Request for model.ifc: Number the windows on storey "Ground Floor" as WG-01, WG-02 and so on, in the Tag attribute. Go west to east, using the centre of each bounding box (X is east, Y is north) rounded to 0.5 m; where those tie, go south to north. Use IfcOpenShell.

First a look at what the model holds.

```python
import ifcopenshell
import ifcopenshell.util.element
import ifcopenshell.util.placement

model = ifcopenshell.open("model.ifc")
print(model.schema)
storey = next(s for s in model.by_type("IfcBuildingStorey") if s.Name == "Ground Floor")
windows = [e for e in ifcopenshell.util.element.get_decomposition(storey) if e.is_a("IfcWindow")]
for e in sorted(windows, key=lambda e: e.id()):
    origin = ifcopenshell.util.placement.get_local_placement(e.ObjectPlacement)[:3, 3]
    print(e.id(), e.Tag, e.Name, origin.round(2) + 0.0, sep=" | ")
```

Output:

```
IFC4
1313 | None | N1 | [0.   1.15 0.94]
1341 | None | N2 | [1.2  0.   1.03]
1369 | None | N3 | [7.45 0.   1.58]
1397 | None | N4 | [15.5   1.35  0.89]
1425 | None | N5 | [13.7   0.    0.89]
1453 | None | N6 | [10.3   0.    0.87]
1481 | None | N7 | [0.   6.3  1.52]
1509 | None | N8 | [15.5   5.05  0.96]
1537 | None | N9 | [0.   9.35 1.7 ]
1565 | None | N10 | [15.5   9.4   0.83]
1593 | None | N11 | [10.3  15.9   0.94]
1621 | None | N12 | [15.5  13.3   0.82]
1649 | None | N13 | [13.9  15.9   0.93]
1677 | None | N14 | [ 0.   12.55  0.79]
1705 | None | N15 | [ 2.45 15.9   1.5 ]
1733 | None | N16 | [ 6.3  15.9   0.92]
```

```python
import ifcopenshell
import ifcopenshell.geom
import ifcopenshell.util.element
import ifcopenshell.util.shape

model = ifcopenshell.open("model.ifc")
settings = ifcopenshell.geom.settings()
settings.set("use-world-coords", True)


def centre(element):
    shape = ifcopenshell.geom.create_shape(settings, element)
    return ifcopenshell.util.shape.get_bbox_centroid(shape.geometry)


storey = next(s for s in model.by_type("IfcBuildingStorey") if s.Name == "Ground Floor")
windows = [e for e in ifcopenshell.util.element.get_decomposition(storey) if e.is_a("IfcWindow")]

# Insertion points can sit at a corner or the storey origin, so sort by the geometry (in metres).
centres = {e: centre(e) for e in windows}
windows.sort(key=lambda e: (round(centres[e][0] / 0.5), centres[e][1]))

for i, e in enumerate(windows, start=1):
    number = f"WG-{i:02d}"
    e.Tag = number
    print(e.id(), number)

model.write("model-out.ifc")
```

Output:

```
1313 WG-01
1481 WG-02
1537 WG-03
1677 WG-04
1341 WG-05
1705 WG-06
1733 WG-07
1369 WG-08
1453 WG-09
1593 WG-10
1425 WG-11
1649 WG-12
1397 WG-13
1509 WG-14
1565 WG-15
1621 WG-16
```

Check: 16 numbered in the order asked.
